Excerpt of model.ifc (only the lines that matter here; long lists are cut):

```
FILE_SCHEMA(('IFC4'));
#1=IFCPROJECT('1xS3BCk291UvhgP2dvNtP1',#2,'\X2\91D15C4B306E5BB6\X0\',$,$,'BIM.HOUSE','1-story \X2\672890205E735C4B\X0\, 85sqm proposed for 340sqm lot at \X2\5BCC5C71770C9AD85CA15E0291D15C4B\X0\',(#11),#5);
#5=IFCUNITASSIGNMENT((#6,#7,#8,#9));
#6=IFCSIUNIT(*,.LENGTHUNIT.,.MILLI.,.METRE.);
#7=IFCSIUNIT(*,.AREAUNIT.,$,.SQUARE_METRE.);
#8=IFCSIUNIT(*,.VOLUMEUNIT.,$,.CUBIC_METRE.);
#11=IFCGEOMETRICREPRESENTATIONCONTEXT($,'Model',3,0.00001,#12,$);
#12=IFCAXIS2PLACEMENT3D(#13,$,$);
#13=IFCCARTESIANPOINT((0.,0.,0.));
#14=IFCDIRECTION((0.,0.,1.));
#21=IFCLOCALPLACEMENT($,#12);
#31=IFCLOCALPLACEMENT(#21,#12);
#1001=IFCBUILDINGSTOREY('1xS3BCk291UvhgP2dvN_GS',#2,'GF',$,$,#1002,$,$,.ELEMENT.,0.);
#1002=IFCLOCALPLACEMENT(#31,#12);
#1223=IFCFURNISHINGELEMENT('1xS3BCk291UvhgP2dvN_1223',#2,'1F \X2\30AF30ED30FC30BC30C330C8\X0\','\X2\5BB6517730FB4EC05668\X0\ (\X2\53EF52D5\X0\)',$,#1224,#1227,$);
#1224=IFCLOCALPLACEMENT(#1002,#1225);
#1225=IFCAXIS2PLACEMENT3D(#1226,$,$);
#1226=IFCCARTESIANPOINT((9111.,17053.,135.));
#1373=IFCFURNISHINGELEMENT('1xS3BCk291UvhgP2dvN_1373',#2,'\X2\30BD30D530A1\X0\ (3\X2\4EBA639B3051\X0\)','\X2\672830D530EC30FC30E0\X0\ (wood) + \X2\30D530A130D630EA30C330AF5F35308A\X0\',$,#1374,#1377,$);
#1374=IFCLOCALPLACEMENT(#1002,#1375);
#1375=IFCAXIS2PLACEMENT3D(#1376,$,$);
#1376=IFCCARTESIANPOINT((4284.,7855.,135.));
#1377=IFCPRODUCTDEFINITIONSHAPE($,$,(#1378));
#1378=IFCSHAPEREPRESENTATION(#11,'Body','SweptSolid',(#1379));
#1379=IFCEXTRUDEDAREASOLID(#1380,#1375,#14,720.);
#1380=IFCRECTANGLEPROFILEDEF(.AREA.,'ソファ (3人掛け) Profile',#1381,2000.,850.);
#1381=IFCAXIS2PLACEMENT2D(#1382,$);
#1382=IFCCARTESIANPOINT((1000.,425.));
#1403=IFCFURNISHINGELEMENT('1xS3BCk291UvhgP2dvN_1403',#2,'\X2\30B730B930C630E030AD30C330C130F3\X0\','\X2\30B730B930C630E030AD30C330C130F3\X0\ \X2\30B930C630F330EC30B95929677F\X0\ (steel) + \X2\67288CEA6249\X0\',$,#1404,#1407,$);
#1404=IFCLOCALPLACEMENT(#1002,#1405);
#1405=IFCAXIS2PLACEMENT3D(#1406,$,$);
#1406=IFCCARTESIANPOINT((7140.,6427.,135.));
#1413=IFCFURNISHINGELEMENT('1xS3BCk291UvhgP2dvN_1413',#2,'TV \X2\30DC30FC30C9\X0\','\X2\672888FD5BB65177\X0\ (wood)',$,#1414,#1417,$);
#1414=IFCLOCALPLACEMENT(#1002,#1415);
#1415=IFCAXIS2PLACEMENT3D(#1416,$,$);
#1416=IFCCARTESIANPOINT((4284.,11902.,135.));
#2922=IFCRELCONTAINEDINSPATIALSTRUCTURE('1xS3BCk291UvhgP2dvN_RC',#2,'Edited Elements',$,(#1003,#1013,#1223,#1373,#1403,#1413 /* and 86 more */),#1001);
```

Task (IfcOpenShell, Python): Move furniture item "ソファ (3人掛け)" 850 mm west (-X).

```python
import ifcopenshell
import ifcopenshell.api.geometry
import ifcopenshell.util.placement

model = ifcopenshell.open("model.ifc")

item = model.by_guid("1xS3BCk291UvhgP2dvN_1373")
matrix = ifcopenshell.util.placement.get_local_placement(item.ObjectPlacement)
matrix[0, 3] -= 850.0
ifcopenshell.api.geometry.edit_object_placement(model, product=item, matrix=matrix, is_si=False)

print(ifcopenshell.util.placement.get_local_placement(item.ObjectPlacement).round(3) + 0.0)

model.write("model_edited.ifc")
```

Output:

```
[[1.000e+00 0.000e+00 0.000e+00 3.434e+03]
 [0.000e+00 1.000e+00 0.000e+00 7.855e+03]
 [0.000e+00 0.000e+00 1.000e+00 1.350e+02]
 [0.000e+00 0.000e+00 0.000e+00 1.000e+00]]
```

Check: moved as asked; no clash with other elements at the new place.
